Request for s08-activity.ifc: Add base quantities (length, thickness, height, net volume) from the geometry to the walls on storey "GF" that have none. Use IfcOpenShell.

First a look at what the model holds.

```python
import ifcopenshell
import ifcopenshell.util.element
import ifcopenshell.util.unit

model = ifcopenshell.open("s08-activity.ifc")
print(model.schema)
for unit_type in ("LENGTHUNIT", "AREAUNIT", "VOLUMEUNIT"):
    print(unit_type, ifcopenshell.util.unit.calculate_unit_scale(model, unit_type))
storey = next(s for s in model.by_type("IfcBuildingStorey") if s.Name == "GF")
walls = [e for e in ifcopenshell.util.element.get_decomposition(storey) if e.is_a("IfcWall")]
for e in sorted(walls, key=lambda e: e.id()):
    print(e.id(), e.is_a(), e.Name, list(ifcopenshell.util.element.get_psets(e, qtos_only=True)), sep=" | ")
```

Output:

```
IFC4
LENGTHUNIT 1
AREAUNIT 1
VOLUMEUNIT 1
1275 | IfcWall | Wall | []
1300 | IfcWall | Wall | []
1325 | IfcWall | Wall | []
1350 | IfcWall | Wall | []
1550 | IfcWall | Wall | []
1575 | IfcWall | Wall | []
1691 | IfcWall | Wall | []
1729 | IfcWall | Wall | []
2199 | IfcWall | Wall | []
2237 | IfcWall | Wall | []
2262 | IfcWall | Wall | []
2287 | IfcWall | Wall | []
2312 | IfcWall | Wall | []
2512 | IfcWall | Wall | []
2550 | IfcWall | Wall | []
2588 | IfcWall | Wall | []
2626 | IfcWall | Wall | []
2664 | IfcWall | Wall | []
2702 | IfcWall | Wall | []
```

```python
import ifcopenshell
import ifcopenshell.api.pset
import ifcopenshell.geom
import ifcopenshell.util.element
import ifcopenshell.util.shape
import ifcopenshell.util.unit

model = ifcopenshell.open("s08-activity.ifc")
unit_scale = ifcopenshell.util.unit.calculate_unit_scale(model)
volume_scale = ifcopenshell.util.unit.calculate_unit_scale(model, "VOLUMEUNIT")
settings = ifcopenshell.geom.settings()

storey = next(s for s in model.by_type("IfcBuildingStorey") if s.Name == "GF")
walls = [e for e in ifcopenshell.util.element.get_decomposition(storey) if e.is_a("IfcWall")]

for e in sorted(walls, key=lambda e: e.id()):
    if ifcopenshell.util.element.get_psets(e, qtos_only=True, should_inherit=False):
        continue
    # Geometry comes back in metres, in the element's own axes.
    shape = ifcopenshell.geom.create_shape(settings, e)
    values = {
        "Length": ifcopenshell.util.shape.get_x(shape.geometry) / unit_scale,
        "Width": ifcopenshell.util.shape.get_y(shape.geometry) / unit_scale,
        "Height": ifcopenshell.util.shape.get_z(shape.geometry) / unit_scale,
        "NetVolume": ifcopenshell.util.shape.get_volume(shape.geometry) / volume_scale,
    }
    qto = ifcopenshell.api.pset.add_qto(model, product=e, name="Qto_WallBaseQuantities")
    ifcopenshell.api.pset.edit_qto(model, qto=qto, properties=values)
    print(e.id(), {k: round(v, 3) for k, v in values.items()})

model.write("s08-activity_updated.ifc")
```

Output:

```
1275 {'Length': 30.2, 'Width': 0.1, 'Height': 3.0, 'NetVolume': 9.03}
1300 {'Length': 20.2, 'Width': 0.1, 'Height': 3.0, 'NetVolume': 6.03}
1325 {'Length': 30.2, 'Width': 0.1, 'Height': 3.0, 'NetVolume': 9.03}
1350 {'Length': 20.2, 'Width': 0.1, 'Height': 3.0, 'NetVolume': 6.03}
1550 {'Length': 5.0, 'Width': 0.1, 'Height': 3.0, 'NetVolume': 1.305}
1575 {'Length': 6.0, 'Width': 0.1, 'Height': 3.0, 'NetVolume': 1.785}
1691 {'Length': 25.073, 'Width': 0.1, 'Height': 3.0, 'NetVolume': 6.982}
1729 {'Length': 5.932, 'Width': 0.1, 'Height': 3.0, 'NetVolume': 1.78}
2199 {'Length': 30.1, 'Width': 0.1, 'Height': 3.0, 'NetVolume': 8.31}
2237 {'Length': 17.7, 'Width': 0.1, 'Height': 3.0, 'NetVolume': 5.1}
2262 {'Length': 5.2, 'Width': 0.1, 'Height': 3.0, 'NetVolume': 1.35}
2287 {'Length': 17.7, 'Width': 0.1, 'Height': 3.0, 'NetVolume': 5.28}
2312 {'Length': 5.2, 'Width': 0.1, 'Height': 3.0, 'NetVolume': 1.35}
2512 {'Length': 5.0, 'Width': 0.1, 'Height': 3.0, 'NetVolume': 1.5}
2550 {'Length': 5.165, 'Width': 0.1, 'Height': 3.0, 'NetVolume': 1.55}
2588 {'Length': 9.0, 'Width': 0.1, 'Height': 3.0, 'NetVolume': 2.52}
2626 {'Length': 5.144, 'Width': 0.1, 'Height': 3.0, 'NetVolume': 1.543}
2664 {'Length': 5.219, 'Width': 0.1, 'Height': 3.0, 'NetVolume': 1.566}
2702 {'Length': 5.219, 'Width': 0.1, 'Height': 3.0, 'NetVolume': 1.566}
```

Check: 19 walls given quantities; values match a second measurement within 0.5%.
